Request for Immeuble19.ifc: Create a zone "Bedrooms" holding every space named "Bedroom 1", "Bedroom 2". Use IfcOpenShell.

First a look at what the model holds.

```python
import ifcopenshell

model = ifcopenshell.open("Immeuble19.ifc")
print(model.schema)
seen = {}
for space in model.by_type("IfcSpace"):
    seen[space.LongName] = seen.get(space.LongName, 0) + 1
for name, count in sorted(seen.items(), key=str):
    print(count, "x", name)
print("zones:", [z.Name for z in model.by_type("IfcZone")][:20])
```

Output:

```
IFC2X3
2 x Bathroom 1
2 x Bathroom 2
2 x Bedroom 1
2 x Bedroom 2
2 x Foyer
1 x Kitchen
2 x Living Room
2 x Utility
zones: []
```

```python
import ifcopenshell
import ifcopenshell.api.group
import ifcopenshell.api.root

model = ifcopenshell.open("Immeuble19.ifc")

names = {"Bedroom 1", "Bedroom 2"}
spaces = [s for s in model.by_type("IfcSpace") if s.LongName in names]

zone = ifcopenshell.api.root.create_entity(model, ifc_class="IfcZone", name="Bedrooms")
ifcopenshell.api.group.assign_group(model, products=spaces, group=zone)
print(len(spaces), "spaces in", zone.Name)

model.write("Immeuble19-out.ifc")
```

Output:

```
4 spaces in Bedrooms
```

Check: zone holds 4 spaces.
